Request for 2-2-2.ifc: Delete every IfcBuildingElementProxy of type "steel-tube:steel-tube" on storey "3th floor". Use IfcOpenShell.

First a look at what the model holds.

```python
import ifcopenshell
import ifcopenshell.util.element

model = ifcopenshell.open("2-2-2.ifc")
print(model.schema)
storey = next(s for s in model.by_type("IfcBuildingStorey") if s.Name == "3th floor")
proxies = [e for e in ifcopenshell.util.element.get_decomposition(storey) if e.is_a("IfcBuildingElementProxy")]
seen = {}
for e in proxies:
    element_type = ifcopenshell.util.element.get_type(e)
    name = element_type.Name if element_type not in (None, e) else None
    seen[name] = seen.get(name, 0) + 1
for name, count in sorted(seen.items(), key=str):
    print(count, "x", name)
```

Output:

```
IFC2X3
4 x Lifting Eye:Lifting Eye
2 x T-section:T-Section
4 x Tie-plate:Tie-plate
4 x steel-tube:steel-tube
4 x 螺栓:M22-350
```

```python
import ifcopenshell
import ifcopenshell.api.root
import ifcopenshell.util.element

model = ifcopenshell.open("2-2-2.ifc")

storey = next(s for s in model.by_type("IfcBuildingStorey") if s.Name == "3th floor")
proxies = [e for e in ifcopenshell.util.element.get_decomposition(storey) if e.is_a("IfcBuildingElementProxy")]
targets = [e for e in proxies if (t := ifcopenshell.util.element.get_type(e)) not in (None, e) and t.Name == "steel-tube:steel-tube"]

for e in targets:
    ifcopenshell.api.root.remove_product(model, product=e)
print(len(targets), "removed")

model.write("2-2-2_edited.ifc")
```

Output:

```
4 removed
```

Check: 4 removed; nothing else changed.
